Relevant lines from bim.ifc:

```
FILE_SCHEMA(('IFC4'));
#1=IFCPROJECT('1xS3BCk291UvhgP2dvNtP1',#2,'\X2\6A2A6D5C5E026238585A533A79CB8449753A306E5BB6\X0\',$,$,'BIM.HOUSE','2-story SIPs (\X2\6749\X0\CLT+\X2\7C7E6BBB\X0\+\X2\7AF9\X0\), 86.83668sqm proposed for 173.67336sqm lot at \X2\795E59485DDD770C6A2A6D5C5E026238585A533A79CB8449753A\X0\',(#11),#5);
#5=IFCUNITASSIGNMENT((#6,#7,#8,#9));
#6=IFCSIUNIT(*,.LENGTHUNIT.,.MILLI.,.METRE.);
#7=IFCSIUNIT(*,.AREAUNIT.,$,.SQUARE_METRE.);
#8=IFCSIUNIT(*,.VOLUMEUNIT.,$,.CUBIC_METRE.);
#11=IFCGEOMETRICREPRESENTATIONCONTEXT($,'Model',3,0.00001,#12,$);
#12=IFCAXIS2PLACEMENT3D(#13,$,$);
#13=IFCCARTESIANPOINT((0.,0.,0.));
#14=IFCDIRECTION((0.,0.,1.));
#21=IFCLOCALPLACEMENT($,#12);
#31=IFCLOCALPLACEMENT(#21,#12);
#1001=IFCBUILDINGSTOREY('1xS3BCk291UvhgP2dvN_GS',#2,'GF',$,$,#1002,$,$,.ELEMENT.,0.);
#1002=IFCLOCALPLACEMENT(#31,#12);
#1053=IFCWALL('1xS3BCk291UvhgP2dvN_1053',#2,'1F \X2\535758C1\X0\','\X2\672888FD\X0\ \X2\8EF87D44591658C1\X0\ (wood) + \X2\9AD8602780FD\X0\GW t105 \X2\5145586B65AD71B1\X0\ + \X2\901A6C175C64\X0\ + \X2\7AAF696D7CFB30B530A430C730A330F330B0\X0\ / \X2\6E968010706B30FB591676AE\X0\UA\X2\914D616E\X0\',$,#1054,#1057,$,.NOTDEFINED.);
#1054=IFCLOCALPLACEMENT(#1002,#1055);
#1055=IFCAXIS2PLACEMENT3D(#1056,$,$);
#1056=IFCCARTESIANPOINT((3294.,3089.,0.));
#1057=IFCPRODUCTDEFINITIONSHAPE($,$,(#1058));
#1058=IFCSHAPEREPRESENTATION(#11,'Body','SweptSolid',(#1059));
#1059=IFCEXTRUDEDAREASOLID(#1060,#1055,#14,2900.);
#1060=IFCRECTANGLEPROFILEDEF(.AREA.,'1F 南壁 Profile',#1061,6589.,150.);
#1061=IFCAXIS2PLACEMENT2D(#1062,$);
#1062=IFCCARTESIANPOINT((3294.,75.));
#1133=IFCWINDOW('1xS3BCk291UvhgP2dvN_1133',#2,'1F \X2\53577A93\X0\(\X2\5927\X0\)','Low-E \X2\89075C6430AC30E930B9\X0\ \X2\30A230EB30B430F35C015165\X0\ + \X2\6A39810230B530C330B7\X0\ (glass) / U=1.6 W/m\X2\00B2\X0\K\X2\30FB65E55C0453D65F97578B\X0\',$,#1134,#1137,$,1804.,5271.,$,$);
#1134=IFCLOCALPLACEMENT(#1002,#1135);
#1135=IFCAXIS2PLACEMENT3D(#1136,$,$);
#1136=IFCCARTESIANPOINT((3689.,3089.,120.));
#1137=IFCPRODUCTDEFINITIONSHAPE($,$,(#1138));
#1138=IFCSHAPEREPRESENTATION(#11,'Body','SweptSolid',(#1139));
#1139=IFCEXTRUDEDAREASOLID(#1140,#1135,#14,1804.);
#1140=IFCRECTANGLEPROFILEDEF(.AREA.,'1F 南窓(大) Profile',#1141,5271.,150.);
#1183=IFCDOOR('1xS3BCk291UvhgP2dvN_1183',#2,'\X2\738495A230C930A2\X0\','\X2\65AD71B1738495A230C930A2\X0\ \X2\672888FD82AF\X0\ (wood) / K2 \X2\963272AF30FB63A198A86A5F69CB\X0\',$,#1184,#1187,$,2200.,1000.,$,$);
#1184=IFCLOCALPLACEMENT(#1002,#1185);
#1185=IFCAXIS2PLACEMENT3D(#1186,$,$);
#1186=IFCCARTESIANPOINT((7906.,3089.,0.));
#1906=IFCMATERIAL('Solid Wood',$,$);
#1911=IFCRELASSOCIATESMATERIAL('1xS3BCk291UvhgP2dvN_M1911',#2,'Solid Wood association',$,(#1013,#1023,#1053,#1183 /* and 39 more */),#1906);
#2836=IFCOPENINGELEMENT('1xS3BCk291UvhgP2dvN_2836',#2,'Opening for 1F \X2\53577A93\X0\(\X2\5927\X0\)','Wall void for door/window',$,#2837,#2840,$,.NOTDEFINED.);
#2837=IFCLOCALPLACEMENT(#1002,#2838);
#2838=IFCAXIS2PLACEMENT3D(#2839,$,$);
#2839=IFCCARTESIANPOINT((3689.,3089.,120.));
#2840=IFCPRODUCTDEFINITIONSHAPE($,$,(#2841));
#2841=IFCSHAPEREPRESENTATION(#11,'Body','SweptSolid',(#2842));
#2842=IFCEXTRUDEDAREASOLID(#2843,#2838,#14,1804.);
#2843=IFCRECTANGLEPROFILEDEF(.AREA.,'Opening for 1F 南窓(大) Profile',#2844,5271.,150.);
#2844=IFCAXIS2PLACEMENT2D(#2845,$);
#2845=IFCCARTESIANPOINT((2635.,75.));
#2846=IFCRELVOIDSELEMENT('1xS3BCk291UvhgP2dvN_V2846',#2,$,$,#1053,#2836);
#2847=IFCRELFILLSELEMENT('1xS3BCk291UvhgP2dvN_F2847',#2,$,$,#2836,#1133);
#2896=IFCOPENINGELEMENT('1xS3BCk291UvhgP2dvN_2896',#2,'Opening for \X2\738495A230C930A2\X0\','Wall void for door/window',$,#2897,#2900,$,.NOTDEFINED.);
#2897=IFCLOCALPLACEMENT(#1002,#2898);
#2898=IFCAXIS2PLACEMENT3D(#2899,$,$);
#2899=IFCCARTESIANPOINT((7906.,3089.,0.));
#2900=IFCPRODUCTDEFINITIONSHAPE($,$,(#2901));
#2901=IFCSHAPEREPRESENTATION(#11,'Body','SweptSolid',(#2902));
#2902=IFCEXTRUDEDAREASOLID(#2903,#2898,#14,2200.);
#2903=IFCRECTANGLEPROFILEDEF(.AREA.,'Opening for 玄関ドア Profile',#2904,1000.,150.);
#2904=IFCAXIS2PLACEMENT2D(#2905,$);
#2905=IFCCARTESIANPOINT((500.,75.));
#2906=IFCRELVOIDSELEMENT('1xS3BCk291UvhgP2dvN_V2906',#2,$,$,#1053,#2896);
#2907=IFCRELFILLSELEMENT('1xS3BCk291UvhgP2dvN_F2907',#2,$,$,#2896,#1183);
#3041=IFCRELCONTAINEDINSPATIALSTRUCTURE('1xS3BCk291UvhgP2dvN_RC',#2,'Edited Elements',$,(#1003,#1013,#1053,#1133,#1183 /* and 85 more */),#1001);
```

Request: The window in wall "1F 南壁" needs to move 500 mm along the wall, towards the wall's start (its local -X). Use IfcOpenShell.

```python
import ifcopenshell
import ifcopenshell.api.geometry
import ifcopenshell.util.placement
import ifcopenshell.util.unit

model = ifcopenshell.open("bim.ifc")
unit_scale = ifcopenshell.util.unit.calculate_unit_scale(model)

window = model.by_guid("1xS3BCk291UvhgP2dvN_1133")
opening = window.FillsVoids[0].RelatingOpeningElement
wall = opening.VoidsElements[0].RelatingBuildingElement

wall_matrix = ifcopenshell.util.placement.get_local_placement(wall.ObjectPlacement)
shift = wall_matrix[:3, 0] * -0.5 / unit_scale
before = ifcopenshell.util.placement.get_local_placement(window.ObjectPlacement)[:3, 3].copy()

# The window is not placed relative to its opening, so move both.
for product in (opening, window):
    matrix = ifcopenshell.util.placement.get_local_placement(product.ObjectPlacement)
    matrix[:3, 3] += shift
    ifcopenshell.api.geometry.edit_object_placement(model, product=product, matrix=matrix, is_si=False)

after = ifcopenshell.util.placement.get_local_placement(window.ObjectPlacement)[:3, 3]
print("window moved by", (after - before).round(3) + 0.0)

model.write("bim_updated.ifc")
```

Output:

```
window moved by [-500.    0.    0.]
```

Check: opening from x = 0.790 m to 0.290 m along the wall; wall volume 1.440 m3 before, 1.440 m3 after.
